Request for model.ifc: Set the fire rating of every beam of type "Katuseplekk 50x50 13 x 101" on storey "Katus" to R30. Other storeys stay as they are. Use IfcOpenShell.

First a look at what the model holds.

```python
import ifcopenshell
import ifcopenshell.util.element

model = ifcopenshell.open("model.ifc")
print(model.schema)
storey = next(s for s in model.by_type("IfcBuildingStorey") if s.Name == "Katus")
beams = [e for e in ifcopenshell.util.element.get_decomposition(storey) if e.is_a("IfcBeam")]
seen = {}
for e in beams:
    element_type = ifcopenshell.util.element.get_type(e)
    key = (element_type.Name if element_type != e and element_type else None, ifcopenshell.util.element.get_pset(e, "Pset_BeamCommon", "FireRating"))
    seen[key] = seen.get(key, 0) + 1
for (name, value), count in sorted(seen.items(), key=str):
    print(count, "x", name, "|", value)
```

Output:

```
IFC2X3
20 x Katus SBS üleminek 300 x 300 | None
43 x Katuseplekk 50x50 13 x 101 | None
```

```python
import ifcopenshell
import ifcopenshell.api.pset
import ifcopenshell.util.element

model = ifcopenshell.open("model.ifc")

storey = next(s for s in model.by_type("IfcBuildingStorey") if s.Name == "Katus")
beams = [e for e in ifcopenshell.util.element.get_decomposition(storey) if e.is_a("IfcBeam")]

count = 0
for e in beams:
    element_type = ifcopenshell.util.element.get_type(e)
    if element_type in (None, e) or element_type.Name != "Katuseplekk 50x50 13 x 101":
        continue
    # add_pset returns the element's existing set when there is one.
    pset = ifcopenshell.api.pset.add_pset(model, product=e, name="Pset_BeamCommon")
    ifcopenshell.api.pset.edit_pset(model, pset=pset, properties={"FireRating": "R30"})
    count += 1

print(count, "beams updated")

model.write("model-out.ifc")
```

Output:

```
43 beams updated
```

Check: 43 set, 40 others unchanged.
